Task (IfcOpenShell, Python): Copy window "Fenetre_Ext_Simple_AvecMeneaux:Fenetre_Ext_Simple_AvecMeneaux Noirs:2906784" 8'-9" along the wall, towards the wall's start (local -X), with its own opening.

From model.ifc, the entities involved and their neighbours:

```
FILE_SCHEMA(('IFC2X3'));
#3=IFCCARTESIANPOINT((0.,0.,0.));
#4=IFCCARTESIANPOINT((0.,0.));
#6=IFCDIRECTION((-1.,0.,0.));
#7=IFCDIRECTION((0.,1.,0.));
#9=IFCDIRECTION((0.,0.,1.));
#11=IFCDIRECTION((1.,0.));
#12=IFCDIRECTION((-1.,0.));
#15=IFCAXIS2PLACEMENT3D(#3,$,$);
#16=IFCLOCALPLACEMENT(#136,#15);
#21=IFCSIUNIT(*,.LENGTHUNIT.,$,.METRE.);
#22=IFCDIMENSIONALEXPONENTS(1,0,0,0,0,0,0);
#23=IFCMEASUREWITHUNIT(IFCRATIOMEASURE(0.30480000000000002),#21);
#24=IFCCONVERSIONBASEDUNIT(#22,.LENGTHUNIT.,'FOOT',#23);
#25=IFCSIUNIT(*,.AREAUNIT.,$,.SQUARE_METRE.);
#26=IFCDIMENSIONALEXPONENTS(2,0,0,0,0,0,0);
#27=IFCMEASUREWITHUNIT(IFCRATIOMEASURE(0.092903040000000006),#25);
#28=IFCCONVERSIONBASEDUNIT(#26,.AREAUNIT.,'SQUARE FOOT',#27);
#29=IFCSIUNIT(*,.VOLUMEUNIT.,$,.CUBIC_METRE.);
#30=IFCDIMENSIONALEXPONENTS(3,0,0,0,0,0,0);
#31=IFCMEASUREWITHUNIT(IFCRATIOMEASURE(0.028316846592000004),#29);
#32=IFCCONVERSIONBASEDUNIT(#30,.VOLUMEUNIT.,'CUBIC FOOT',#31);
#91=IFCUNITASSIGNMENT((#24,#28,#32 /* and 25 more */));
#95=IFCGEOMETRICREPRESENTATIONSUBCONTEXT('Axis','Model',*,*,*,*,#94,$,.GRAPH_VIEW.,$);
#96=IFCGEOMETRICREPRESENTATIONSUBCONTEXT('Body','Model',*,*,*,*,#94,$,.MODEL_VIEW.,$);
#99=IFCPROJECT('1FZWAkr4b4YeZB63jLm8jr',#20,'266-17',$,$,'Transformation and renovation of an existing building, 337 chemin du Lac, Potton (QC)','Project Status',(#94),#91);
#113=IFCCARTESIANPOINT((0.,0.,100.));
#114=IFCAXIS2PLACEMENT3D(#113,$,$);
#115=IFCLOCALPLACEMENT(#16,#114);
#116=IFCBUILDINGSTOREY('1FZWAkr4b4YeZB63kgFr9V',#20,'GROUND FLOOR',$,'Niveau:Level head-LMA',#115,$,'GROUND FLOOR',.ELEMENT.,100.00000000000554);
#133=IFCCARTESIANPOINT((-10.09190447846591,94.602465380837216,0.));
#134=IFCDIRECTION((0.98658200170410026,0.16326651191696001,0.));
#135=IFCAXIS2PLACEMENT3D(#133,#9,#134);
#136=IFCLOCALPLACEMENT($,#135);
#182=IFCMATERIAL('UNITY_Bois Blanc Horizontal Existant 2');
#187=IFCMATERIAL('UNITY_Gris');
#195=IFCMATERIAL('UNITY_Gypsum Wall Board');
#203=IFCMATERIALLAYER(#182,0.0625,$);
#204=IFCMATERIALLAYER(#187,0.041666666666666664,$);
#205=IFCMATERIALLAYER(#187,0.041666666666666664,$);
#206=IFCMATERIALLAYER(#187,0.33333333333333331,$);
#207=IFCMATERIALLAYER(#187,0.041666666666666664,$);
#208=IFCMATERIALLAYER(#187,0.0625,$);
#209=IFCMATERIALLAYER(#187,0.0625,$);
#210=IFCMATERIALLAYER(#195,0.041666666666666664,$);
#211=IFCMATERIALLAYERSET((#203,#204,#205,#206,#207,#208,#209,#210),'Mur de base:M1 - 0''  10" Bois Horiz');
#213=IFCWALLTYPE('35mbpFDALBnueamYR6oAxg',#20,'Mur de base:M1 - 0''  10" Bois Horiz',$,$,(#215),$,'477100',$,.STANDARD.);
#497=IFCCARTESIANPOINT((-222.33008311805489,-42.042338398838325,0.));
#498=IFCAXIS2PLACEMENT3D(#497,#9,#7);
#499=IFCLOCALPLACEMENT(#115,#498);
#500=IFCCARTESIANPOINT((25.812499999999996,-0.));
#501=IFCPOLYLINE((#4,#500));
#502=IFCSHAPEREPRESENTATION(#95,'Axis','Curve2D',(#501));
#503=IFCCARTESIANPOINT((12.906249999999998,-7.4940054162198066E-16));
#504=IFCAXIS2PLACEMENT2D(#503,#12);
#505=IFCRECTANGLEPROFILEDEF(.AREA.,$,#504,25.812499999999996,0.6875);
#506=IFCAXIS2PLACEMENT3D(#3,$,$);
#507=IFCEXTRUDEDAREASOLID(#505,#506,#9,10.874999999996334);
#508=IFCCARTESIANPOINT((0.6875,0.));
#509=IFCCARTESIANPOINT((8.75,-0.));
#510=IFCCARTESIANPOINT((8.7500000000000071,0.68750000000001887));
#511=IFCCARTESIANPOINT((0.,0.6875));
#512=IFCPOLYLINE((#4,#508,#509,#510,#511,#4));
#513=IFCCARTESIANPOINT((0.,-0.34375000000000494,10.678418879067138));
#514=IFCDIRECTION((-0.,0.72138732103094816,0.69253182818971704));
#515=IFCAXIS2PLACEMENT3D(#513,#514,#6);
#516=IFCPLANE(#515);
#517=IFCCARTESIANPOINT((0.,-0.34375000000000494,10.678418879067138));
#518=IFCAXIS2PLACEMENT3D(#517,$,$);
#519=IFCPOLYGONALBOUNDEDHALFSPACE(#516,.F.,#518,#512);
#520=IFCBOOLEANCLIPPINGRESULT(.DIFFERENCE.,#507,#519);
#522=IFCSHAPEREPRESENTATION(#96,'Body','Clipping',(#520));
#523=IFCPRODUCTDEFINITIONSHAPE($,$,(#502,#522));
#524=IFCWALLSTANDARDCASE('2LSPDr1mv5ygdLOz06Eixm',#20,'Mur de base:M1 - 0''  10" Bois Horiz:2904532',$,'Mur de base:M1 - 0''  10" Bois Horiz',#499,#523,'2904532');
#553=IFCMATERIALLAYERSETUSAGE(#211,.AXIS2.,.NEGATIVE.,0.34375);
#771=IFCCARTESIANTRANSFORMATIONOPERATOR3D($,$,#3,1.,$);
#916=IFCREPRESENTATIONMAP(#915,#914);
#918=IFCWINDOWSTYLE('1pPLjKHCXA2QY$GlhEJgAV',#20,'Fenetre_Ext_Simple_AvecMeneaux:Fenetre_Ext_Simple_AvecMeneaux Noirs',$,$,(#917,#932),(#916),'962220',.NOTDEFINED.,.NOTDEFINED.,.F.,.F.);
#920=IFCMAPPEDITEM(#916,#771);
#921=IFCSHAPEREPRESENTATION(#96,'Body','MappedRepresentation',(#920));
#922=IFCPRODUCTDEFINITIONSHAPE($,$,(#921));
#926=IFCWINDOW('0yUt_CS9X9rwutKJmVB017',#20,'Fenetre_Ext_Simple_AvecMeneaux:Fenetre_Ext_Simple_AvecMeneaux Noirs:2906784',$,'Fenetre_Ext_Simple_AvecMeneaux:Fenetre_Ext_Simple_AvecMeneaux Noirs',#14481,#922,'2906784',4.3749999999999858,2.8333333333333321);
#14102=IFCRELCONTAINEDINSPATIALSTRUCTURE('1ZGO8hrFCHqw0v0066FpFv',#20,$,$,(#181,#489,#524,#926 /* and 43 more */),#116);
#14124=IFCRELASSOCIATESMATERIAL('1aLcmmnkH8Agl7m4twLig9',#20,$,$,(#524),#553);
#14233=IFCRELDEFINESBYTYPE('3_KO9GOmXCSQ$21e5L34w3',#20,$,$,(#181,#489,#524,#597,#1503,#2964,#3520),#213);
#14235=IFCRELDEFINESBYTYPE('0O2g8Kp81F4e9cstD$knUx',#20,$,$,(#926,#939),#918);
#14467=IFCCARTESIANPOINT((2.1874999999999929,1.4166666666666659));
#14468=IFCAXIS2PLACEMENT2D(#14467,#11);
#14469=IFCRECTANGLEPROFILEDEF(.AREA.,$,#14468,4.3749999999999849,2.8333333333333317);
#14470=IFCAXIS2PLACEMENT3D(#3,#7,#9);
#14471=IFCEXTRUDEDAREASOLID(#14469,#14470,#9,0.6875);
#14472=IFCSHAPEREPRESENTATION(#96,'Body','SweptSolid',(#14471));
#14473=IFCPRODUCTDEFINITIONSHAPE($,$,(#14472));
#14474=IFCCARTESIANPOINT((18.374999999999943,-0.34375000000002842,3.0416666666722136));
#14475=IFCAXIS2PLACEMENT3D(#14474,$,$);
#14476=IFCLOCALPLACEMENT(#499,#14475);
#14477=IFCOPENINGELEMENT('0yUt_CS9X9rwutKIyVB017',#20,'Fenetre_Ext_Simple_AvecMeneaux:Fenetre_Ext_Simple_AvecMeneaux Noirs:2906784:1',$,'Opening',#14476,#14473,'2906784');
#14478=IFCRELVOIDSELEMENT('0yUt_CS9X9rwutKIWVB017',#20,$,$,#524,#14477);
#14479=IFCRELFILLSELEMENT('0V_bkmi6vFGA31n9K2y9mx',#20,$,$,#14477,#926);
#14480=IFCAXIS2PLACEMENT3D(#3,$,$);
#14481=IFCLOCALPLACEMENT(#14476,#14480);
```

```python
import ifcopenshell
import ifcopenshell.api.feature
import ifcopenshell.api.geometry
import ifcopenshell.api.root
import ifcopenshell.geom
import ifcopenshell.util.element
import ifcopenshell.util.placement
import ifcopenshell.util.shape
import ifcopenshell.util.unit

model = ifcopenshell.open("model.ifc")
unit_scale = ifcopenshell.util.unit.calculate_unit_scale(model)
settings = ifcopenshell.geom.settings()


def volume(element):
    """Net volume in cubic metres, openings subtracted."""
    shape = ifcopenshell.geom.create_shape(settings, element)
    return ifcopenshell.util.shape.get_volume(shape.geometry)


def reuse_history(source, copy):
    """copy_class also copies each property set's owner history, people and application; keep the originals."""
    for rel in copy.IsDefinedBy:
        if rel.is_a("IfcRelDefinesByProperties") and (history := rel.RelatingPropertyDefinition.OwnerHistory):
            rel.RelatingPropertyDefinition.OwnerHistory = source.OwnerHistory
            ifcopenshell.util.element.remove_deep2(model, history)


window = model.by_id(926)
opening = window.FillsVoids[0].RelatingOpeningElement
wall = opening.VoidsElements[0].RelatingBuildingElement
before = volume(wall)
shift = ifcopenshell.util.placement.get_local_placement(wall.ObjectPlacement)[:3, 0] * -105 * 0.0254 / unit_scale

# copy_class copies the void relationship, type, container and properties, but no geometry.
new_opening = ifcopenshell.api.root.copy_class(model, product=opening)
new_opening.Representation = ifcopenshell.util.element.copy_deep(
    model, opening.Representation, exclude=["IfcGeometricRepresentationContext", "IfcRepresentationMap"]
)
new_opening.Name = "Fenetre_Ext_Simple_AvecMeneaux:Fenetre_Ext_Simple_AvecMeneaux Noirs"
new_opening.Tag = None
new_window = ifcopenshell.api.root.copy_class(model, product=window)
new_window.Representation = ifcopenshell.util.element.copy_deep(
    model, window.Representation, exclude=["IfcGeometricRepresentationContext", "IfcRepresentationMap"]
)
new_window.Name = "Fenetre_Ext_Simple_AvecMeneaux:Fenetre_Ext_Simple_AvecMeneaux Noirs"
new_window.Tag = None
reuse_history(window, new_window)
fills = ifcopenshell.api.feature.add_filling(model, opening=new_opening, element=new_window)
fills.OwnerHistory = new_window.OwnerHistory  # required in IFC2X3

for old, new in ((opening, new_opening), (window, new_window)):
    matrix = ifcopenshell.util.placement.get_local_placement(old.ObjectPlacement)
    matrix[:3, 3] += shift
    ifcopenshell.api.geometry.edit_object_placement(model, product=new, matrix=matrix, is_si=False)

after = volume(wall)

print(f"wall volume {before:.3f} -> {after:.3f} m3")

model.write("model_edited.ifc")
```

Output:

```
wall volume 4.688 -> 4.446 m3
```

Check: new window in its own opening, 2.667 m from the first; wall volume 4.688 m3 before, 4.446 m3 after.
